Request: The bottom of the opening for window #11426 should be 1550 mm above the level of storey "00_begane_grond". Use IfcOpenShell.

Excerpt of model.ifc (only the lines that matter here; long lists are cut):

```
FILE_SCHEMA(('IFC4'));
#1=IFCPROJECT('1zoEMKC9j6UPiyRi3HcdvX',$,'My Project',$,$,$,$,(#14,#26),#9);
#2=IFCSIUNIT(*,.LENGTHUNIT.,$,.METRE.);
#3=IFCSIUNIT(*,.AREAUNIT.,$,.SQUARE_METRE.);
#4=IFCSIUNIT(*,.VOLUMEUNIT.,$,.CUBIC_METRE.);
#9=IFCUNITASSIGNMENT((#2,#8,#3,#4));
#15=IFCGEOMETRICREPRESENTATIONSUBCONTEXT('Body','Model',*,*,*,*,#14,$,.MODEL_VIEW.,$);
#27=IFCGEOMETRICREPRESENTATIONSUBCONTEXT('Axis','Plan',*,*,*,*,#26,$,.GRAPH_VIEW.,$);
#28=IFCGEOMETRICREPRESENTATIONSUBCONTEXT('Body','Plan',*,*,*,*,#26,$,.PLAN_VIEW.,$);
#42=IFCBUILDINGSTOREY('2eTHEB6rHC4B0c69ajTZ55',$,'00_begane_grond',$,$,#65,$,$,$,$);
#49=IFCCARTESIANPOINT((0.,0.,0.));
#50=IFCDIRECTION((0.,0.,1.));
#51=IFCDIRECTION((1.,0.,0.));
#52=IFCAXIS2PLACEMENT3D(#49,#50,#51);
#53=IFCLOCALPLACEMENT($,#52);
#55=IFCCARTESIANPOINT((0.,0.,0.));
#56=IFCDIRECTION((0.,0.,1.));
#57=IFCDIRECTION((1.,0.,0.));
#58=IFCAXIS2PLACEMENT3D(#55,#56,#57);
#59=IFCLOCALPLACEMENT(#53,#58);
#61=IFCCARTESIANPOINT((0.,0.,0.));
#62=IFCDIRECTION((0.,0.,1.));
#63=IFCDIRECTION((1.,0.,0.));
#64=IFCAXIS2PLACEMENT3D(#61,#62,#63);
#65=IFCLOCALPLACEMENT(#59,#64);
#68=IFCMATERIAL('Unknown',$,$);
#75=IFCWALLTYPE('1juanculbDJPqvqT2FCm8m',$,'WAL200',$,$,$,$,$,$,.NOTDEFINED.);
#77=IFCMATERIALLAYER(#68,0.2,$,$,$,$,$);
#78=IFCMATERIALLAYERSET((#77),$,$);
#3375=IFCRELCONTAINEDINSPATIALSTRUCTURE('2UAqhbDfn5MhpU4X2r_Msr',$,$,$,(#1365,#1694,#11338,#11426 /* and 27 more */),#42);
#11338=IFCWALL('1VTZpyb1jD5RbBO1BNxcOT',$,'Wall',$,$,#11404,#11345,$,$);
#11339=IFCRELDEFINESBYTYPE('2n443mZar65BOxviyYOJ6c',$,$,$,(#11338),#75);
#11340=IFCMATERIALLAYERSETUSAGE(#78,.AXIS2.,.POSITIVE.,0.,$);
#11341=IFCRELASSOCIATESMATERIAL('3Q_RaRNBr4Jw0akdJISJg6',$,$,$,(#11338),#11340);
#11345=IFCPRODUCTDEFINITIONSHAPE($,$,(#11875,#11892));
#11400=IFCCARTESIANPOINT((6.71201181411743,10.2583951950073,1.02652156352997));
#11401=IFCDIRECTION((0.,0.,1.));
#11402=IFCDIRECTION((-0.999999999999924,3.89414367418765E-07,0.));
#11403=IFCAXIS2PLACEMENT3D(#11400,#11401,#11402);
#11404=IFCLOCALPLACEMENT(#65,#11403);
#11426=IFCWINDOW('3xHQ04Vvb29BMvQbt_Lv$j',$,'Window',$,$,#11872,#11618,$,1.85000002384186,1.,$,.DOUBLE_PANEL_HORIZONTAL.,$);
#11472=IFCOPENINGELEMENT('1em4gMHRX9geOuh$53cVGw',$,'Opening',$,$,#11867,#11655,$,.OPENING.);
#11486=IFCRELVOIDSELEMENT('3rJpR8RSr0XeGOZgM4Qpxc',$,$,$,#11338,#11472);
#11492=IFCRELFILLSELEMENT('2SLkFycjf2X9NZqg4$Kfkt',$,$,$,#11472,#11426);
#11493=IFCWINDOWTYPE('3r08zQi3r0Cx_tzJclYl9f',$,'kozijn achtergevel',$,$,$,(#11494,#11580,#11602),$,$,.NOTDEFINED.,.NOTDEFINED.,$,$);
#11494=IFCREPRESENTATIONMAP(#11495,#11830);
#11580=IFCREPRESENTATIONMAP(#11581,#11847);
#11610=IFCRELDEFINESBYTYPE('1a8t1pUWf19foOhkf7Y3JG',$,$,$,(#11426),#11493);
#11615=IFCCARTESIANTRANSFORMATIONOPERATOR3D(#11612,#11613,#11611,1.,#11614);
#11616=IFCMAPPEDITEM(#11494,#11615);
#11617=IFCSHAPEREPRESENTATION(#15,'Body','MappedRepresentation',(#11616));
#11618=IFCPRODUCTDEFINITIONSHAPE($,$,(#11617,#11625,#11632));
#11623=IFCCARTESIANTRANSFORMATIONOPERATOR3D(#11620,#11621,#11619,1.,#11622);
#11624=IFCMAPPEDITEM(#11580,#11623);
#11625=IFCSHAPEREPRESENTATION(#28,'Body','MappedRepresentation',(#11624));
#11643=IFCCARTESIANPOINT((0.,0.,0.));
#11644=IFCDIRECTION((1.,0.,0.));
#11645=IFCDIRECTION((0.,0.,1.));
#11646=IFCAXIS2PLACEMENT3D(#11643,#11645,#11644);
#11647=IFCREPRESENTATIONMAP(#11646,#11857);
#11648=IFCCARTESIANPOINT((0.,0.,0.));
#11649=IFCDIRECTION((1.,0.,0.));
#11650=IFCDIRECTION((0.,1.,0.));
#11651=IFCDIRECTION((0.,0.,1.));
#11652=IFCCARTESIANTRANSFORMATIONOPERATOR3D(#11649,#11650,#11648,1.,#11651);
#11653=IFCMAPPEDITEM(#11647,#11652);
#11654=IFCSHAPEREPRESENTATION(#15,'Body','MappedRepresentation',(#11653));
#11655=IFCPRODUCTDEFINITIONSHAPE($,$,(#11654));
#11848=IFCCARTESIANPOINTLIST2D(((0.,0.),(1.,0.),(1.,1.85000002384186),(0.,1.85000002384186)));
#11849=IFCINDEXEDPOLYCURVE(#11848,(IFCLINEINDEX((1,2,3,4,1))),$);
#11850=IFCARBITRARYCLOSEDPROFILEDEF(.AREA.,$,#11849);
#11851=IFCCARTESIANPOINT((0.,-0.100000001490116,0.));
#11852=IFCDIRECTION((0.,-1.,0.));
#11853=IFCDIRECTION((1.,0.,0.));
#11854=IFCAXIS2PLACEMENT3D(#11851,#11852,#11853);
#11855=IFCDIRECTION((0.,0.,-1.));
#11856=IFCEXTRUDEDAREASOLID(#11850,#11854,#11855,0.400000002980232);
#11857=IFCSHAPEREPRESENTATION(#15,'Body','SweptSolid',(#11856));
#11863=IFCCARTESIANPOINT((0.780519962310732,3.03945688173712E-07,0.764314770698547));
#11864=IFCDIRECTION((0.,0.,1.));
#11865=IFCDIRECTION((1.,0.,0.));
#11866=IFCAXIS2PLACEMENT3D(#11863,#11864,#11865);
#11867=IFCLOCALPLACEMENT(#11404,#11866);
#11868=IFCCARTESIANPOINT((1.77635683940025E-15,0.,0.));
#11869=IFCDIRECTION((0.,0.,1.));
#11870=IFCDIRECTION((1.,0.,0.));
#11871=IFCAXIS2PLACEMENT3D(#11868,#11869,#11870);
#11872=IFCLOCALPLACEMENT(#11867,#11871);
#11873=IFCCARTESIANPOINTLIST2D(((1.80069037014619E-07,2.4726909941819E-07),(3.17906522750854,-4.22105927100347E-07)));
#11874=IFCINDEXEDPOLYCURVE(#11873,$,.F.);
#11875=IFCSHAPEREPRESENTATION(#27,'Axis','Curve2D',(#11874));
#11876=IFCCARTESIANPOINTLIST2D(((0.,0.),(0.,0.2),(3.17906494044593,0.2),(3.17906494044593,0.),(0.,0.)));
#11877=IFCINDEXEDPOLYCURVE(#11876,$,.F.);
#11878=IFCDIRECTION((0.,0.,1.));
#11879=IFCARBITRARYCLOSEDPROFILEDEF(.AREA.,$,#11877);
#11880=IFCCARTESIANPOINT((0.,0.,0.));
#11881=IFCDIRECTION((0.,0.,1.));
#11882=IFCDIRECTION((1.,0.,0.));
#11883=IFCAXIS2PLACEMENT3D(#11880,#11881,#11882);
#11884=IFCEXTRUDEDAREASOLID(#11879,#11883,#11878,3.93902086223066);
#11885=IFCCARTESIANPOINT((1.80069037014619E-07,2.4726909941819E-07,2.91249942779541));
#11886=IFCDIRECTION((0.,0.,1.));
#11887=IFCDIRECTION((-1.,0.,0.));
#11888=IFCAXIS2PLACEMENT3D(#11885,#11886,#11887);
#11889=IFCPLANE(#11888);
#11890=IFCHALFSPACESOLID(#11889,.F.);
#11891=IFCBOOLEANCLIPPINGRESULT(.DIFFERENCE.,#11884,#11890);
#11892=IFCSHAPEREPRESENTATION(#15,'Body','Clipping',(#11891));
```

```python
import numpy as np
import ifcopenshell
import ifcopenshell.api.geometry
import ifcopenshell.geom
import ifcopenshell.util.element
import ifcopenshell.util.placement
import ifcopenshell.util.shape
import ifcopenshell.util.unit

model = ifcopenshell.open("model.ifc")
unit_scale = ifcopenshell.util.unit.calculate_unit_scale(model)

window = model.by_guid("3xHQ04Vvb29BMvQbt_Lv$j")
opening = window.FillsVoids[0].RelatingOpeningElement
storey = ifcopenshell.util.element.get_container(window, ifc_class="IfcBuildingStorey")
level = ifcopenshell.util.placement.get_local_placement(storey.ObjectPlacement)[2, 3]

# The opening's origin need not be at the sill, so measure its lowest point.
shape = ifcopenshell.geom.create_shape(ifcopenshell.geom.settings(), opening)
bottom = ifcopenshell.util.shape.get_shape_bottom_elevation(shape, shape.geometry) / unit_scale
dz = level + 1.55 - bottom

shift = np.array([0.0, 0.0, dz])
# The window is placed relative to its opening, so it follows when the opening moves.
matrix = ifcopenshell.util.placement.get_local_placement(opening.ObjectPlacement)
matrix[:3, 3] += shift
ifcopenshell.api.geometry.edit_object_placement(
    model, product=opening, matrix=matrix, is_si=False, should_transform_children=True
)

print(f"moved by {dz * unit_scale:+.3f} m")

model.write("model_rev.ifc")
```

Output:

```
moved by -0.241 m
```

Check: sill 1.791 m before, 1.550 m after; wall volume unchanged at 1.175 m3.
